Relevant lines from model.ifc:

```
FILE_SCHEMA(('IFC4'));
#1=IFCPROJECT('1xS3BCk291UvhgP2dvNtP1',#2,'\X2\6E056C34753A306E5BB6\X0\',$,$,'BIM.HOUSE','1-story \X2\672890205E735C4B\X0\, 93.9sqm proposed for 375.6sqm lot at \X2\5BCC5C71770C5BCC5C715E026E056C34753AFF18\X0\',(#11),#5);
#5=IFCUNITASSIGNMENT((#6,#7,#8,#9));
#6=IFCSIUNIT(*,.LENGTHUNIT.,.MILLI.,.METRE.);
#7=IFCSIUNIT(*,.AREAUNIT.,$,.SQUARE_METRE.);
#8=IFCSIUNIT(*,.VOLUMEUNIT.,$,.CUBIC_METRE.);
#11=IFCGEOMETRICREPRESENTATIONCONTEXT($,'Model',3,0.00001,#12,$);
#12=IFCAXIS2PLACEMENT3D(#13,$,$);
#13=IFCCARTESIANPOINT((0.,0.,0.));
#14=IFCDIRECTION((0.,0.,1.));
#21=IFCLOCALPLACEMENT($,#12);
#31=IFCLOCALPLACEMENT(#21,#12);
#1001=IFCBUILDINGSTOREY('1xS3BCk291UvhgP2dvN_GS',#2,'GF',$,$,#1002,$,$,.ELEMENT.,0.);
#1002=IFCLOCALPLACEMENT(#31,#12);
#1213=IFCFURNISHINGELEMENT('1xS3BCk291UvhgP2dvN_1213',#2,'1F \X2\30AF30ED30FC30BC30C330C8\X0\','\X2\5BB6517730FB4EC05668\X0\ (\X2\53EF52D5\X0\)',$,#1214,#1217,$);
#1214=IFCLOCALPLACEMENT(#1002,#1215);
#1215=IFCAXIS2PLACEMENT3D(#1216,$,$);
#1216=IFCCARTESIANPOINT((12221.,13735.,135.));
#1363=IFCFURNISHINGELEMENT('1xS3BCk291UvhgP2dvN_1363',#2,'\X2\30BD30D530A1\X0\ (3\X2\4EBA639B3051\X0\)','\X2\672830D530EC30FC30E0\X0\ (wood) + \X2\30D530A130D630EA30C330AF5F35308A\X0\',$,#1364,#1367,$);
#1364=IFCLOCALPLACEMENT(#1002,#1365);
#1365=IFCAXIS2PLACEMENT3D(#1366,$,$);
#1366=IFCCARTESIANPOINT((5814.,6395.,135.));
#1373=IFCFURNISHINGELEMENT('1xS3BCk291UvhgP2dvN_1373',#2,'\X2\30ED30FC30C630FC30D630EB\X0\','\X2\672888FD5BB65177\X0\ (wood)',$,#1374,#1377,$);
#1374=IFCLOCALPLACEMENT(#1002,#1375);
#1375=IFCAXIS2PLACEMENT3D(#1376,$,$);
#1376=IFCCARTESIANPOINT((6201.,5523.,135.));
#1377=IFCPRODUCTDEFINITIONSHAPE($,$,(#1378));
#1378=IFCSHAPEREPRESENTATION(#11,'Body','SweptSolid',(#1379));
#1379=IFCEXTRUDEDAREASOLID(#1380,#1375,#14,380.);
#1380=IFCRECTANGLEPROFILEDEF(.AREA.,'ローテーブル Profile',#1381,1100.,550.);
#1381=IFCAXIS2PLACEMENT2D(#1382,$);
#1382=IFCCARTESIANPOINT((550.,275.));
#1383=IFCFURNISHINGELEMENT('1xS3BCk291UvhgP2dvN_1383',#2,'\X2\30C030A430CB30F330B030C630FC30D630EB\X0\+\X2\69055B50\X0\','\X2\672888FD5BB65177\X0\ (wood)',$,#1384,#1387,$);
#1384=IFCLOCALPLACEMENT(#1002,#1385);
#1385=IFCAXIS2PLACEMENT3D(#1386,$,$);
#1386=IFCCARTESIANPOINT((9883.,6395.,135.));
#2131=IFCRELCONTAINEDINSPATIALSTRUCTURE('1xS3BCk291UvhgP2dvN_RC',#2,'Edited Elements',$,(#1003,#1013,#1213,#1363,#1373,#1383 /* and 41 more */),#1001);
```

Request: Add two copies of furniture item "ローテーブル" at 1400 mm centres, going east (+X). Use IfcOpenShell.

```python
import numpy as np
import ifcopenshell
import ifcopenshell.api.geometry
import ifcopenshell.api.root
import ifcopenshell.util.element
import ifcopenshell.util.placement
import ifcopenshell.util.unit

model = ifcopenshell.open("model.ifc")
unit_scale = ifcopenshell.util.unit.calculate_unit_scale(model)


def reuse_history(source, copy):
    """copy_class also copies each property set's owner history, people and application; keep the originals."""
    for rel in copy.IsDefinedBy:
        if rel.is_a("IfcRelDefinesByProperties") and (history := rel.RelatingPropertyDefinition.OwnerHistory):
            rel.RelatingPropertyDefinition.OwnerHistory = source.OwnerHistory
            ifcopenshell.util.element.remove_deep2(model, history)


source = model.by_guid("1xS3BCk291UvhgP2dvN_1373")
base = ifcopenshell.util.placement.get_local_placement(source.ObjectPlacement)
step = np.array([1.0, 0.0, 0.0]) * 1.4 / unit_scale

for i in range(1, 3):
    copy = ifcopenshell.api.root.copy_class(model, product=source)
    copy.Representation = ifcopenshell.util.element.copy_deep(
        model, source.Representation, exclude=["IfcGeometricRepresentationContext", "IfcRepresentationMap"]
    )
    reuse_history(source, copy)
    matrix = base.copy()
    matrix[:3, 3] += i * step
    print("added at", matrix[:3, 3].round(3) + 0.0)
    ifcopenshell.api.geometry.edit_object_placement(model, product=copy, matrix=matrix, is_si=False)

model.write("model_edited.ifc")
```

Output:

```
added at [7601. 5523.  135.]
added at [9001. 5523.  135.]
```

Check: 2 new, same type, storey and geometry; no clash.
